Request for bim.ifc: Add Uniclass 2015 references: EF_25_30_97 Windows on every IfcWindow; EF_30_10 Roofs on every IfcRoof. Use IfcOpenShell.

First a look at what the model holds.

```python
import ifcopenshell

model = ifcopenshell.open("bim.ifc")
print(model.schema)
print("classifications:", [c.Name for c in model.by_type("IfcClassification")])
for ifc_class in ("IfcDoor", "IfcRoof", "IfcStair", "IfcWall", "IfcWindow"):
    print(ifc_class, len(model.by_type(ifc_class)))
```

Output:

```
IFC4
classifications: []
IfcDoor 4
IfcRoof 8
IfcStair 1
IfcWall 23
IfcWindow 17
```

```python
import ifcopenshell
import ifcopenshell.api.classification

model = ifcopenshell.open("bim.ifc")

system = ifcopenshell.api.classification.add_classification(model, classification="Uniclass 2015")

codes = {
    "IfcWindow": ("EF_25_30_97", "Windows"),
    "IfcRoof": ("EF_30_10", "Roofs"),
}
for ifc_class, (code, name) in codes.items():
    products = model.by_type(ifc_class)
    ifcopenshell.api.classification.add_reference(
        model, products=products, classification=system, identification=code, name=name
    )
    print(code, len(products))

model.write("bim_updated.ifc")
```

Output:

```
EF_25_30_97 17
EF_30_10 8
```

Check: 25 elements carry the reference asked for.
